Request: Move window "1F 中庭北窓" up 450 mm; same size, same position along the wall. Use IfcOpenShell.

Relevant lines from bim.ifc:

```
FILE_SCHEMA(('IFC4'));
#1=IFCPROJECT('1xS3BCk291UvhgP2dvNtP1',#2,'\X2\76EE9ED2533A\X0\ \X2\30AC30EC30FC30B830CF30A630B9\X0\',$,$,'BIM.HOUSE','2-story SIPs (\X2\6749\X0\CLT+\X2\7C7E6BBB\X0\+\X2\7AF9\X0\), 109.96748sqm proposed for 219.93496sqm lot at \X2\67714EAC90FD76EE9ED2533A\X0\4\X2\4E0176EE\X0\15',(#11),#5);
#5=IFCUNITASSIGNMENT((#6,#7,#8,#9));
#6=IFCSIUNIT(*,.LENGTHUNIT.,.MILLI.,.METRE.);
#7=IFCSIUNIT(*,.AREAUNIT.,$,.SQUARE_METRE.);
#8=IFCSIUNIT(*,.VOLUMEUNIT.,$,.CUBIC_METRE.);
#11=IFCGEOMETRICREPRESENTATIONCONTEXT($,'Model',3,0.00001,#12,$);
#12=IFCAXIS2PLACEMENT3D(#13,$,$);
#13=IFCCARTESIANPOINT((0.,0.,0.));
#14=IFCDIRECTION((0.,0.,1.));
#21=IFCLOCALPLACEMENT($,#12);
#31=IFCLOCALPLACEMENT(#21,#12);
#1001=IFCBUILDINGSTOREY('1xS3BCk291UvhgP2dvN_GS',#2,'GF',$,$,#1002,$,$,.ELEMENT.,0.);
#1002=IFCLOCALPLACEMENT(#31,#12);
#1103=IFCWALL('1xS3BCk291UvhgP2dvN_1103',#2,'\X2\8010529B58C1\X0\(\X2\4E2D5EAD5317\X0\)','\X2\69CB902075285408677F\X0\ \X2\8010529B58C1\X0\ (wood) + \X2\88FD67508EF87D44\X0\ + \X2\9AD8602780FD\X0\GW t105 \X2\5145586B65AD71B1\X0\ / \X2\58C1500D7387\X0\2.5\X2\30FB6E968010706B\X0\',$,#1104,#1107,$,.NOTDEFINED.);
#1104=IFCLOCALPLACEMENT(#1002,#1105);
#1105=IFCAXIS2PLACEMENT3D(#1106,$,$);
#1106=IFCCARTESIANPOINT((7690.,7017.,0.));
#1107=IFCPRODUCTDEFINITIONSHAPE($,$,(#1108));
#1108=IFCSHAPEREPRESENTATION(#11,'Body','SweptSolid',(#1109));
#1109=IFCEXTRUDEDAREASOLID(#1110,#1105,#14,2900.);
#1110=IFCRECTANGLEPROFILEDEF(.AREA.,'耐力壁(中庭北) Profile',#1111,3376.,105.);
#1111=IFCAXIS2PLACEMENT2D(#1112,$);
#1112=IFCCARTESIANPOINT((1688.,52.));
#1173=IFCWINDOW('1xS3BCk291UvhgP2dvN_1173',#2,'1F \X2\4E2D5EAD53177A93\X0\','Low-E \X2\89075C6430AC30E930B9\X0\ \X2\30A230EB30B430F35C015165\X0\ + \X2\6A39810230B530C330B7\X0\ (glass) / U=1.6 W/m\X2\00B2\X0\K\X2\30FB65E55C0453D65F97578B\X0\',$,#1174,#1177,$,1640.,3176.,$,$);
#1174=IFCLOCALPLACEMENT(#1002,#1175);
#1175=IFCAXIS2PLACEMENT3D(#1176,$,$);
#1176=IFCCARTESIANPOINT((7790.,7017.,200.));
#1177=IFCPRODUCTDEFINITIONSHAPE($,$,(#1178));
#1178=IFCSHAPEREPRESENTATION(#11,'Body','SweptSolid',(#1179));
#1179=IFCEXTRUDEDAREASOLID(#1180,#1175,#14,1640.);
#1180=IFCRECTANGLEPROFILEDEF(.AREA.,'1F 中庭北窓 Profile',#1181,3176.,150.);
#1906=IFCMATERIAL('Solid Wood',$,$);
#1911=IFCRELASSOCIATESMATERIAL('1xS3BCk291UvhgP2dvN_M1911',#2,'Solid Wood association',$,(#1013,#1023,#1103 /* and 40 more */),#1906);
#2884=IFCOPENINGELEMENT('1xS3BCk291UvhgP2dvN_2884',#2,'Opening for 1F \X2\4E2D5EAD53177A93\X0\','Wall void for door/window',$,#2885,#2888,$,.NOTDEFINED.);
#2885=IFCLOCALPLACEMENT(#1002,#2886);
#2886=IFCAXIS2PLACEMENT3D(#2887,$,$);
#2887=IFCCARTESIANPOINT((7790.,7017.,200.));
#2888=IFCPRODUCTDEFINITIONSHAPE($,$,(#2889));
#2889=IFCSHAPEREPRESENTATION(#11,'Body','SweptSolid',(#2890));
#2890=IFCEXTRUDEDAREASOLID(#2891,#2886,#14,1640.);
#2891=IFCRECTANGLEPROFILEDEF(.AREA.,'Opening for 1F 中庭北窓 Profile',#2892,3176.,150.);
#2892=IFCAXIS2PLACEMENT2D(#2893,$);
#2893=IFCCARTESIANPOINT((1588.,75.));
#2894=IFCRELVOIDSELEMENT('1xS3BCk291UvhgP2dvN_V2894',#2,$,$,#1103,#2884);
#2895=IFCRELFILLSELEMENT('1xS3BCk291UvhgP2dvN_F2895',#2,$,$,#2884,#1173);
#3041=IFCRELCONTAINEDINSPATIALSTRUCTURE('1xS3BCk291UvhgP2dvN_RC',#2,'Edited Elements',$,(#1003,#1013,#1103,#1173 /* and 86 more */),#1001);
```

```python
import numpy as np
import ifcopenshell
import ifcopenshell.api.geometry
import ifcopenshell.util.placement
import ifcopenshell.util.unit

model = ifcopenshell.open("bim.ifc")
unit_scale = ifcopenshell.util.unit.calculate_unit_scale(model)

window = model.by_guid("1xS3BCk291UvhgP2dvN_1173")
opening = window.FillsVoids[0].RelatingOpeningElement
dz = 0.45 / unit_scale

shift = np.array([0.0, 0.0, dz])
# The window is not placed relative to its opening, so move both.
for product in (opening, window):
    matrix = ifcopenshell.util.placement.get_local_placement(product.ObjectPlacement)
    matrix[:3, 3] += shift
    ifcopenshell.api.geometry.edit_object_placement(model, product=product, matrix=matrix, is_si=False)

print(f"moved by {dz * unit_scale:+.3f} m")

model.write("bim-out.ifc")
```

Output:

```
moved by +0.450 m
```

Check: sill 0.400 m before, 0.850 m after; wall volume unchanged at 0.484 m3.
